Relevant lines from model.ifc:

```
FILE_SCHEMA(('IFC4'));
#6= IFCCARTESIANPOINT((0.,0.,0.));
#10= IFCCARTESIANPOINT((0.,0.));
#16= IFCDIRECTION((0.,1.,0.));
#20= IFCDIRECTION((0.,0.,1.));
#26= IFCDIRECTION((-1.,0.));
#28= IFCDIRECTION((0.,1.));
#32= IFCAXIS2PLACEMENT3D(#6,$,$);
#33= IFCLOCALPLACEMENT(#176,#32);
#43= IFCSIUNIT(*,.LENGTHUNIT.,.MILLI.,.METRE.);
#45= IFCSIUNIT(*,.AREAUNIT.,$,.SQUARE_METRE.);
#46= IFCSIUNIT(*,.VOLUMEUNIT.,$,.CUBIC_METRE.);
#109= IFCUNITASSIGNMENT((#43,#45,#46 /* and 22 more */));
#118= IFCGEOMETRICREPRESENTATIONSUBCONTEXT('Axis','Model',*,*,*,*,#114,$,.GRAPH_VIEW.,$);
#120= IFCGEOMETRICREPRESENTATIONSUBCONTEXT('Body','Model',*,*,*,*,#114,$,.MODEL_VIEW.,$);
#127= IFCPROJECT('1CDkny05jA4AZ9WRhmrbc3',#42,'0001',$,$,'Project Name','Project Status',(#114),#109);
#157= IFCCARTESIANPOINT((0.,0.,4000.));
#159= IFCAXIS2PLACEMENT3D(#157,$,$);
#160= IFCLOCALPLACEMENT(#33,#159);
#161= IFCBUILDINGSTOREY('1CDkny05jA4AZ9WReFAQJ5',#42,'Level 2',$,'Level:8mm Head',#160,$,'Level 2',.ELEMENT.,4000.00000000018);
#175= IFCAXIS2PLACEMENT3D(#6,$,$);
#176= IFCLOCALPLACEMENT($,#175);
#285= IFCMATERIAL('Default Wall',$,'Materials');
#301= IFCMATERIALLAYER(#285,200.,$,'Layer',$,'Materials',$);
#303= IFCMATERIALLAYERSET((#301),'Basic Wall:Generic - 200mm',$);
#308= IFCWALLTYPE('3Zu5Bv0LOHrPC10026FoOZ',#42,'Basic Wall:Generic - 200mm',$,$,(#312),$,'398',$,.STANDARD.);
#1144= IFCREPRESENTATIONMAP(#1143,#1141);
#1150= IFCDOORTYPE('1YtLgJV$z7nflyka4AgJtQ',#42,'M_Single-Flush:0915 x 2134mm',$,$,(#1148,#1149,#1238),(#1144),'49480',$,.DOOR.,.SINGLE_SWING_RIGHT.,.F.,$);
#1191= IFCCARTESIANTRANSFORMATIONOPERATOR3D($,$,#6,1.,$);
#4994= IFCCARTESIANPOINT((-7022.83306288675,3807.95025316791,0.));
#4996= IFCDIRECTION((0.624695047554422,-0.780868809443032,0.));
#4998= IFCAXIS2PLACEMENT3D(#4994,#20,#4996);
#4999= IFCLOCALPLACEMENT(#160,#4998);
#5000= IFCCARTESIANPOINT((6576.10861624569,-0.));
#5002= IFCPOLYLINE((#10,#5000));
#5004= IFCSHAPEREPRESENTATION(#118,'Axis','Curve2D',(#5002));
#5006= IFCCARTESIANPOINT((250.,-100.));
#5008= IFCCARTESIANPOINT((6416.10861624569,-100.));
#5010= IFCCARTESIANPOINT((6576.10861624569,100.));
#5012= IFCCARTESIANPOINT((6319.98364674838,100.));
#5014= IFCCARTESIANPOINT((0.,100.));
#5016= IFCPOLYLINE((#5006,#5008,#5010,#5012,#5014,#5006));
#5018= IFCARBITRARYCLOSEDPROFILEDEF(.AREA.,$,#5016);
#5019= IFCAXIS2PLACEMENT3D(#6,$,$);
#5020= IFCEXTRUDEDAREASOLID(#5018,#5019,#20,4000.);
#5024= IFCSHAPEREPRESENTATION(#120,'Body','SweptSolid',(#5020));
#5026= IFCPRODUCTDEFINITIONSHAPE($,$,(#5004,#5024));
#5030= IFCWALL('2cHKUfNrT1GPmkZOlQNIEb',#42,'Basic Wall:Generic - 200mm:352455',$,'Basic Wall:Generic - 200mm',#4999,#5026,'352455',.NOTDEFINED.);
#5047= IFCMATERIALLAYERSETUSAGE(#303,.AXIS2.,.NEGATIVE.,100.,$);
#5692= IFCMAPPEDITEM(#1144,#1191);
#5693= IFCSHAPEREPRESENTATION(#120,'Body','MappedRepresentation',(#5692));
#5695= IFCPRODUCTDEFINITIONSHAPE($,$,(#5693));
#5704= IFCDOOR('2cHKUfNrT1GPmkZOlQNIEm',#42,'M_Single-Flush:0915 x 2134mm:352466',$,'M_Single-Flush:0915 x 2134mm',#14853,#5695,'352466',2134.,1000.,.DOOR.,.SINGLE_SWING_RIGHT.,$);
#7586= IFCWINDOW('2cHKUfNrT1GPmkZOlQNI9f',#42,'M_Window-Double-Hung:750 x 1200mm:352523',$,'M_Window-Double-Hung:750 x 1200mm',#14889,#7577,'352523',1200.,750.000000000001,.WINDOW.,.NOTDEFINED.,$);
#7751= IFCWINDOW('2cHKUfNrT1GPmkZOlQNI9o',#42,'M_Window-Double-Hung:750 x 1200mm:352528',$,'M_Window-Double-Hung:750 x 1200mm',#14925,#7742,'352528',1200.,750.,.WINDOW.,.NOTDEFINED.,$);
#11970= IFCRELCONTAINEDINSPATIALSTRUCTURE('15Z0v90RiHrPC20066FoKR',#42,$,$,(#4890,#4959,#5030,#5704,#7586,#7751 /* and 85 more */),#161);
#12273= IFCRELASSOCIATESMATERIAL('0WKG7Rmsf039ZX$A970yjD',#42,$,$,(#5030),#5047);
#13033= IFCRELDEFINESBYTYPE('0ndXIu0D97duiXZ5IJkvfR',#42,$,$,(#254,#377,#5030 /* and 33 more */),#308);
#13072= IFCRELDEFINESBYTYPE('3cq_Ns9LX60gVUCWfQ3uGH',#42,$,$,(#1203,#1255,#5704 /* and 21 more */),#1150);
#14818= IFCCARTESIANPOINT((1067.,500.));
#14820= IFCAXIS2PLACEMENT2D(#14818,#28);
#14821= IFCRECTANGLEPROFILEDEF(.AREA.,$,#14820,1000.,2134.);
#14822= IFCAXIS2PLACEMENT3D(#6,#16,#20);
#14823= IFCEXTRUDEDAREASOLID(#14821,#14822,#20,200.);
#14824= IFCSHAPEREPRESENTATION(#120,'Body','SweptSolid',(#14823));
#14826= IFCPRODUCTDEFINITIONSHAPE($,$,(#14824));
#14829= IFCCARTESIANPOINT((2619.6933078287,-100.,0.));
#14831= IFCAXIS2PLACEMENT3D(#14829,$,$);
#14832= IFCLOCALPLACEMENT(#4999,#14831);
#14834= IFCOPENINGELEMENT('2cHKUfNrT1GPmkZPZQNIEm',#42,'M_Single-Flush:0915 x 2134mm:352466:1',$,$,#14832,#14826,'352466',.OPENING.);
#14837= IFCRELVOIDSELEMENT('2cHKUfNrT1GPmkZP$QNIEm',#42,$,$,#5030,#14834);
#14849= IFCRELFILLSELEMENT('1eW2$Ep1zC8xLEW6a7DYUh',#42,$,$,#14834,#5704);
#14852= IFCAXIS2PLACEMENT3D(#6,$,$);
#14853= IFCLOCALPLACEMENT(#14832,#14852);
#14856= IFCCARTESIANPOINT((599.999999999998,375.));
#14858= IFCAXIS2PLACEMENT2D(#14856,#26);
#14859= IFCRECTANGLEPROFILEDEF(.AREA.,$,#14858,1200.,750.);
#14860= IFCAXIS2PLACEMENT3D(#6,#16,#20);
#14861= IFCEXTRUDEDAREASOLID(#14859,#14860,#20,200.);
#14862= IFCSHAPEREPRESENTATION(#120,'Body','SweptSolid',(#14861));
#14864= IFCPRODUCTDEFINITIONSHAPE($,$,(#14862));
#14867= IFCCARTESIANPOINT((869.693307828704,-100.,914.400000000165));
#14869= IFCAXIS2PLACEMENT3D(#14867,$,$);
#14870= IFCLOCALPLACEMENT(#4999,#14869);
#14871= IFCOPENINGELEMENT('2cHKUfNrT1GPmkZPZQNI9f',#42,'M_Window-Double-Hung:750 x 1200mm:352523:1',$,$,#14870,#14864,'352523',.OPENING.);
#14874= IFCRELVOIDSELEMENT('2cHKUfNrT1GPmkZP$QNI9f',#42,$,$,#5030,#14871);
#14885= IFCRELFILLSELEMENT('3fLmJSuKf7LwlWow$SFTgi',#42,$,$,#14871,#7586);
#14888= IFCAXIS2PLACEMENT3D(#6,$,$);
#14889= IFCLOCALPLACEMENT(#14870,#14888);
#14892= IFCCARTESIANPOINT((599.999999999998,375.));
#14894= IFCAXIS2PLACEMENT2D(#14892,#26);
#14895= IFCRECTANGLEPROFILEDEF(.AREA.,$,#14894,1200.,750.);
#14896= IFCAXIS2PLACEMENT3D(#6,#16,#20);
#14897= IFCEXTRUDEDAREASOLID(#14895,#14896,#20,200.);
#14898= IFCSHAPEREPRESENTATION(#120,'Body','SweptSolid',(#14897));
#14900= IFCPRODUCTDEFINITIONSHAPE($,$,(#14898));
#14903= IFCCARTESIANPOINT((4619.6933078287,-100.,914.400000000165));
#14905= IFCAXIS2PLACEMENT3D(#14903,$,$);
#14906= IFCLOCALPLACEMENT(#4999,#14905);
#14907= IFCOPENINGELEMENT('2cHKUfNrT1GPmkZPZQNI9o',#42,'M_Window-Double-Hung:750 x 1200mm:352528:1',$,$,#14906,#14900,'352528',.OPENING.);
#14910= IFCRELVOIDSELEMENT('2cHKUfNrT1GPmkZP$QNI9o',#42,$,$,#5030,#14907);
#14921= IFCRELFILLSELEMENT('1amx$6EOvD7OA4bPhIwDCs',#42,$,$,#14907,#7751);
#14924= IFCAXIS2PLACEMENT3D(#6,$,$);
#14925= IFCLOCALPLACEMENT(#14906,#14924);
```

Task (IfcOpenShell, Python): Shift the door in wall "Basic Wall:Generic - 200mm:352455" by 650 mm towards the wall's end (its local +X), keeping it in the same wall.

```python
import ifcopenshell
import ifcopenshell.api.geometry
import ifcopenshell.util.placement
import ifcopenshell.util.unit

model = ifcopenshell.open("model.ifc")
unit_scale = ifcopenshell.util.unit.calculate_unit_scale(model)

door = model.by_guid("2cHKUfNrT1GPmkZOlQNIEm")
opening = door.FillsVoids[0].RelatingOpeningElement
wall = opening.VoidsElements[0].RelatingBuildingElement

wall_matrix = ifcopenshell.util.placement.get_local_placement(wall.ObjectPlacement)
shift = wall_matrix[:3, 0] * 0.65 / unit_scale
before = ifcopenshell.util.placement.get_local_placement(door.ObjectPlacement)[:3, 3].copy()

# The door is placed relative to its opening, so it follows when the opening moves.
matrix = ifcopenshell.util.placement.get_local_placement(opening.ObjectPlacement)
matrix[:3, 3] += shift
ifcopenshell.api.geometry.edit_object_placement(
    model, product=opening, matrix=matrix, is_si=False, should_transform_children=True
)

after = ifcopenshell.util.placement.get_local_placement(door.ObjectPlacement)[:3, 3]
print("door moved by", (after - before).round(3) + 0.0)

model.write("model_edited.ifc")
```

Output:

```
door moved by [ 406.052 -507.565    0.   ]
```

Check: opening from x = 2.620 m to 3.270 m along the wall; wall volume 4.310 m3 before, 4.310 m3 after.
